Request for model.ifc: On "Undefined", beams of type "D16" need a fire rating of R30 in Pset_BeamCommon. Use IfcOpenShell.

First a look at what the model holds.

```python
import ifcopenshell
import ifcopenshell.util.element

model = ifcopenshell.open("model.ifc")
print(model.schema)
storey = next(s for s in model.by_type("IfcBuildingStorey") if s.Name == "Undefined")
beams = [e for e in ifcopenshell.util.element.get_decomposition(storey) if e.is_a("IfcBeam")]
seen = {}
for e in beams:
    element_type = ifcopenshell.util.element.get_type(e)
    key = (element_type.Name if element_type != e and element_type else None, ifcopenshell.util.element.get_pset(e, "Pset_BeamCommon", "FireRating"))
    seen[key] = seen.get(key, 0) + 1
for (name, value), count in sorted(seen.items(), key=str):
    print(count, "x", name, "|", value)
```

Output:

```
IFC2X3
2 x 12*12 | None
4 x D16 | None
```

```python
import ifcopenshell
import ifcopenshell.api.pset
import ifcopenshell.util.element

model = ifcopenshell.open("model.ifc")

storey = next(s for s in model.by_type("IfcBuildingStorey") if s.Name == "Undefined")
beams = [e for e in ifcopenshell.util.element.get_decomposition(storey) if e.is_a("IfcBeam")]

count = 0
for e in beams:
    element_type = ifcopenshell.util.element.get_type(e)
    if element_type in (None, e) or element_type.Name != "D16":
        continue
    # add_pset returns the element's existing set when there is one.
    pset = ifcopenshell.api.pset.add_pset(model, product=e, name="Pset_BeamCommon")
    ifcopenshell.api.pset.edit_pset(model, pset=pset, properties={"FireRating": "R30"})
    count += 1

print(count, "beams updated")

model.write("model_updated.ifc")
```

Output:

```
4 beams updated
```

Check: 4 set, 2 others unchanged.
